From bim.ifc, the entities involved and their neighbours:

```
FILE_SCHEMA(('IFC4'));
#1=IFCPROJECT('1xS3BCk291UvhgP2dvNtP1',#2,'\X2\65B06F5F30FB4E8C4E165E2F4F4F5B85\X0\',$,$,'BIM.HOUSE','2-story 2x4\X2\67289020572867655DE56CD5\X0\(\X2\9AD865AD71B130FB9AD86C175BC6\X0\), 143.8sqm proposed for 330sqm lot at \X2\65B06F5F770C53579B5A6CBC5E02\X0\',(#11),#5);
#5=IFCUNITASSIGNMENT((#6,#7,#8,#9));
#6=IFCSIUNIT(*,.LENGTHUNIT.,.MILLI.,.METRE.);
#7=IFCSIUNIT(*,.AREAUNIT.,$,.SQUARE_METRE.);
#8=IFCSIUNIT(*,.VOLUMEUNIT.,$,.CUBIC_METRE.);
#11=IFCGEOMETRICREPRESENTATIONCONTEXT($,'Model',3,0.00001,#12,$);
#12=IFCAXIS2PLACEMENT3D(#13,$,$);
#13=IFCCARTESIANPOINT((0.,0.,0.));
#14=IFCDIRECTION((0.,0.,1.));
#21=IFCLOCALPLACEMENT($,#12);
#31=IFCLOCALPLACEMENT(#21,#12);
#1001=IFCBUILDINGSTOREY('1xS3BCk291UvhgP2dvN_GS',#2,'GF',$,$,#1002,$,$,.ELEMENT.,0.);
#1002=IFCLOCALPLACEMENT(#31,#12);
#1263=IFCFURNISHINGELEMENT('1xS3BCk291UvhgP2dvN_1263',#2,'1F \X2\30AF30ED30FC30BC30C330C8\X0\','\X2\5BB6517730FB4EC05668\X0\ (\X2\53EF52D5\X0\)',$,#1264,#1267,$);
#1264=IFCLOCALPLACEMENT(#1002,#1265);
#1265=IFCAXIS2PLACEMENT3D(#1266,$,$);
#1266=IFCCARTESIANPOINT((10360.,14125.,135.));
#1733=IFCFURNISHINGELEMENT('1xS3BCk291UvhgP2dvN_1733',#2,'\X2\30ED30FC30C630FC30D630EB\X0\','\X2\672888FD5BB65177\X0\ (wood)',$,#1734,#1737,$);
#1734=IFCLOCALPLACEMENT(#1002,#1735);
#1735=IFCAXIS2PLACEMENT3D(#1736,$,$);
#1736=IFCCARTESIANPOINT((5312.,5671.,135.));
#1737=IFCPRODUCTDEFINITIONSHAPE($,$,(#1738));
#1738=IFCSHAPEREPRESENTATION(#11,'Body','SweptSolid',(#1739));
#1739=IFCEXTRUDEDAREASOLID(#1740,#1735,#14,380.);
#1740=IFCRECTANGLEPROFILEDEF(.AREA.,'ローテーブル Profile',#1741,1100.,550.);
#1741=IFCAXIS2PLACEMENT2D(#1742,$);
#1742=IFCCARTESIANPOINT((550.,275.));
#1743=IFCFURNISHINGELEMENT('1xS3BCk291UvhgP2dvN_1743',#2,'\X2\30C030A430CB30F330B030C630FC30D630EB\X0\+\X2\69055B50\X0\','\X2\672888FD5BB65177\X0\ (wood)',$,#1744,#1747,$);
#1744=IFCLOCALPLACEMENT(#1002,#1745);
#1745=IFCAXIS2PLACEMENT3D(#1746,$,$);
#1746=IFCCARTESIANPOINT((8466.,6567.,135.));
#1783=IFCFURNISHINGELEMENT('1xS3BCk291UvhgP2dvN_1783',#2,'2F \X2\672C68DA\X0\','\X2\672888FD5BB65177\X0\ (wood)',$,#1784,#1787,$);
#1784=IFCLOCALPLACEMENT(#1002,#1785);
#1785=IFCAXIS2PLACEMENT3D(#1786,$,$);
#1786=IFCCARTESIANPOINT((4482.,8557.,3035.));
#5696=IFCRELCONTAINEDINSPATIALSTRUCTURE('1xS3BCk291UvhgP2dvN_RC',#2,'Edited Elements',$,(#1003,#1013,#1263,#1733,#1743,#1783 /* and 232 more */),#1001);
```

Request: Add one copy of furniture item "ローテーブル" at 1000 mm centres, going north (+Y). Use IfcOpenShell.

```python
import numpy as np
import ifcopenshell
import ifcopenshell.api.geometry
import ifcopenshell.api.root
import ifcopenshell.util.element
import ifcopenshell.util.placement
import ifcopenshell.util.unit

model = ifcopenshell.open("bim.ifc")
unit_scale = ifcopenshell.util.unit.calculate_unit_scale(model)


def reuse_history(source, copy):
    """copy_class also copies each property set's owner history, people and application; keep the originals."""
    for rel in copy.IsDefinedBy:
        if rel.is_a("IfcRelDefinesByProperties") and (history := rel.RelatingPropertyDefinition.OwnerHistory):
            rel.RelatingPropertyDefinition.OwnerHistory = source.OwnerHistory
            ifcopenshell.util.element.remove_deep2(model, history)


source = model.by_guid("1xS3BCk291UvhgP2dvN_1733")
base = ifcopenshell.util.placement.get_local_placement(source.ObjectPlacement)
step = np.array([0.0, 1.0, 0.0]) * 1 / unit_scale

for i in range(1, 2):
    copy = ifcopenshell.api.root.copy_class(model, product=source)
    copy.Representation = ifcopenshell.util.element.copy_deep(
        model, source.Representation, exclude=["IfcGeometricRepresentationContext", "IfcRepresentationMap"]
    )
    reuse_history(source, copy)
    matrix = base.copy()
    matrix[:3, 3] += i * step
    print("added at", matrix[:3, 3].round(3) + 0.0)
    ifcopenshell.api.geometry.edit_object_placement(model, product=copy, matrix=matrix, is_si=False)

model.write("bim_updated.ifc")
```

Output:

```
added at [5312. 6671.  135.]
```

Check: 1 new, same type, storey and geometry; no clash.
